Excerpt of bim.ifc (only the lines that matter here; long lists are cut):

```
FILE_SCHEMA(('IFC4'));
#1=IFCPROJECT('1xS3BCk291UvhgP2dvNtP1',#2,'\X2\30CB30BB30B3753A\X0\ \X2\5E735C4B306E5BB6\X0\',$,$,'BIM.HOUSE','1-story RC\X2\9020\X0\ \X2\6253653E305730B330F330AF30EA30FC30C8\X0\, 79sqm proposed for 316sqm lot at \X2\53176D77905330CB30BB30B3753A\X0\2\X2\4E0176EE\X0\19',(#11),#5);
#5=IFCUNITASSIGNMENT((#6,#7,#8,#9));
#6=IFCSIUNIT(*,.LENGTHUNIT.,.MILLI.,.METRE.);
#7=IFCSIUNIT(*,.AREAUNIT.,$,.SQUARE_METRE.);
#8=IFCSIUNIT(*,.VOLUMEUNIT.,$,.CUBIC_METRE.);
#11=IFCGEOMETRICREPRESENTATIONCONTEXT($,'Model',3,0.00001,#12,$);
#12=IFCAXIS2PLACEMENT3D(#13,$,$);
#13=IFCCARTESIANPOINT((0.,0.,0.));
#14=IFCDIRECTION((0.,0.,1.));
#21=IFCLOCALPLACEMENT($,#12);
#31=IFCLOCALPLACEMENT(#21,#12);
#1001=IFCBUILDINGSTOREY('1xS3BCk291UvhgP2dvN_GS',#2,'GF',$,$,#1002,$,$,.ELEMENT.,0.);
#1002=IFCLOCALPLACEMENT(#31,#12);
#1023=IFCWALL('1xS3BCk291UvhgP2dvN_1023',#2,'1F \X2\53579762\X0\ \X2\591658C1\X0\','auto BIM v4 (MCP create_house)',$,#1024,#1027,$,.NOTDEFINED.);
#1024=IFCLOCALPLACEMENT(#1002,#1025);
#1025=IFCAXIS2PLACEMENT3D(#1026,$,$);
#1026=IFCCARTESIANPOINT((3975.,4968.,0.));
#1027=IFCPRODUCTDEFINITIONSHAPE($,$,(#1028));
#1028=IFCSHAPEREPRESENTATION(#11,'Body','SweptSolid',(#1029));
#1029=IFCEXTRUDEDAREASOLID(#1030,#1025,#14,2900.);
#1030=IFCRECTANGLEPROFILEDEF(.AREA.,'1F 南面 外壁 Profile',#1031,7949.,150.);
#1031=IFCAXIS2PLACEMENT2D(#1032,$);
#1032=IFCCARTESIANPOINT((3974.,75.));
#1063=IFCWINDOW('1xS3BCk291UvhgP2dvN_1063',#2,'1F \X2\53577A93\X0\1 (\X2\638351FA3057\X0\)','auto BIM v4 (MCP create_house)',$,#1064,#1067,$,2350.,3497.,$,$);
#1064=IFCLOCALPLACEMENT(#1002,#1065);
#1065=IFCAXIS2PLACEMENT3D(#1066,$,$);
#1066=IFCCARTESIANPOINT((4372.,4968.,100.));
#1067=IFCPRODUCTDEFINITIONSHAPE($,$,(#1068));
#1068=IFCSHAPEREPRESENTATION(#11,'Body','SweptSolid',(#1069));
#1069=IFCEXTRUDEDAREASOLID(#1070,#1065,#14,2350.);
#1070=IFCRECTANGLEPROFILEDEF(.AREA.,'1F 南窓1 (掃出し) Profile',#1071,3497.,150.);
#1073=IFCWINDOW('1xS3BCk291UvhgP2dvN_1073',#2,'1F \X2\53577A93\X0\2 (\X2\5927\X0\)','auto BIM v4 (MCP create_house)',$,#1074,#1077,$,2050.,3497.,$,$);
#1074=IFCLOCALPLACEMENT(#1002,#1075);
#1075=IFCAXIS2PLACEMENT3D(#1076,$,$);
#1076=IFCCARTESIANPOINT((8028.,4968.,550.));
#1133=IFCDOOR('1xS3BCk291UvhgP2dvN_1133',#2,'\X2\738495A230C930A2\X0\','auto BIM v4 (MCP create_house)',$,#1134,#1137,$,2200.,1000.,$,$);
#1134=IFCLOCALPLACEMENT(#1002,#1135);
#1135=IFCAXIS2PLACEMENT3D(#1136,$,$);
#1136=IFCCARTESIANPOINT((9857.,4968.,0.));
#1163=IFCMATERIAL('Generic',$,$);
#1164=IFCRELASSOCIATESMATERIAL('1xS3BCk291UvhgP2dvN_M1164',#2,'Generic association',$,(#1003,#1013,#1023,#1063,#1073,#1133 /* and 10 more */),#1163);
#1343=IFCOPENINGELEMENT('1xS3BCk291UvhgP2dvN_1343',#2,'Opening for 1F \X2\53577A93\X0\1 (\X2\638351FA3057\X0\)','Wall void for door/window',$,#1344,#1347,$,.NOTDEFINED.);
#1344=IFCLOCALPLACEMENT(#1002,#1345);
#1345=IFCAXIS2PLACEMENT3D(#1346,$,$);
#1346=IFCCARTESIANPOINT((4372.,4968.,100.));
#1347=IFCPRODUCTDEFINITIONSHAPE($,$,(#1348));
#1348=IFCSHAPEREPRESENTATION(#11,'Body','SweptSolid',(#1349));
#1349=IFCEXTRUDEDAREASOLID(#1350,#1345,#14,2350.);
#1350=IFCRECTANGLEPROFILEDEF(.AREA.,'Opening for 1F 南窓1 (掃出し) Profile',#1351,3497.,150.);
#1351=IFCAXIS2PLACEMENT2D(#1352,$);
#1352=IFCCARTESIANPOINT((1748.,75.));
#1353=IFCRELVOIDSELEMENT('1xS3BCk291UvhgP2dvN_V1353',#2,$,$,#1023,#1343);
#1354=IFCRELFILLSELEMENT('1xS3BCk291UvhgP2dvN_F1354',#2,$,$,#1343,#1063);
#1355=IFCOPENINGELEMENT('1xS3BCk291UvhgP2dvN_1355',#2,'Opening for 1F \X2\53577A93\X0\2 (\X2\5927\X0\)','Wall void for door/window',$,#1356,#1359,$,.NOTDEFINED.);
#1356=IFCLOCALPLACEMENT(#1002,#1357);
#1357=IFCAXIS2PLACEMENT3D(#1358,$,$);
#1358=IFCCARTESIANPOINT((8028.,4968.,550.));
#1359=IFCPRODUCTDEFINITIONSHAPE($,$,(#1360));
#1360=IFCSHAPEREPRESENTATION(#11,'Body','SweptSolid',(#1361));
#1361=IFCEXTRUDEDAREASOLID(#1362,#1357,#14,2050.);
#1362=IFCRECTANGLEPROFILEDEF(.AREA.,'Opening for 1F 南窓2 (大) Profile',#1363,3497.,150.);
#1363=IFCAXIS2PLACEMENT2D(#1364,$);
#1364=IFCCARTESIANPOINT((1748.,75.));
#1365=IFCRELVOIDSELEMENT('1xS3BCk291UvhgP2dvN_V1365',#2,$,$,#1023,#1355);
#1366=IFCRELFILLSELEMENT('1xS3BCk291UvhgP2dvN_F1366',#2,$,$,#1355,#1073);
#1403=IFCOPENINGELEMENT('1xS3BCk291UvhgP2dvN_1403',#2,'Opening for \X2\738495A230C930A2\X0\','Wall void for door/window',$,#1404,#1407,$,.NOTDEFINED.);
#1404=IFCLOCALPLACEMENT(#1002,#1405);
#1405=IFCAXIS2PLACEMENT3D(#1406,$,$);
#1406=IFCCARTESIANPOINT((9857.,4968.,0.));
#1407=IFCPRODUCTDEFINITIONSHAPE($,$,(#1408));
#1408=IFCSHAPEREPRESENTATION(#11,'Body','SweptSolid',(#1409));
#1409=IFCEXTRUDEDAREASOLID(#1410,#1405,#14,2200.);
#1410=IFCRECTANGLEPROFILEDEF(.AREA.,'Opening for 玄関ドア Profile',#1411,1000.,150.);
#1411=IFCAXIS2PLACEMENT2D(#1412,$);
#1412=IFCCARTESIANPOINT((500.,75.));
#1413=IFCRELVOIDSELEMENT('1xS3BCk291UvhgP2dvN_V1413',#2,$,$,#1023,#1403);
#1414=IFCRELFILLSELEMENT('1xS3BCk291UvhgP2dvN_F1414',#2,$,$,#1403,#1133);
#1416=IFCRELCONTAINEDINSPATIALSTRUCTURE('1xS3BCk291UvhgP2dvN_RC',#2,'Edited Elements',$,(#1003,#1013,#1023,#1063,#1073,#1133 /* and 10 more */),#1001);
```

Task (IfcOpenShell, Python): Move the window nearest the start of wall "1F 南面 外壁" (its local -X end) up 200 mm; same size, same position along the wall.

```python
import numpy as np
import ifcopenshell
import ifcopenshell.api.geometry
import ifcopenshell.util.placement
import ifcopenshell.util.unit

model = ifcopenshell.open("bim.ifc")
unit_scale = ifcopenshell.util.unit.calculate_unit_scale(model)

window = model.by_guid("1xS3BCk291UvhgP2dvN_1063")
opening = window.FillsVoids[0].RelatingOpeningElement
dz = 0.2 / unit_scale

shift = np.array([0.0, 0.0, dz])
# The window is not placed relative to its opening, so move both.
for product in (opening, window):
    matrix = ifcopenshell.util.placement.get_local_placement(product.ObjectPlacement)
    matrix[:3, 3] += shift
    ifcopenshell.api.geometry.edit_object_placement(model, product=product, matrix=matrix, is_si=False)

print(f"moved by {dz * unit_scale:+.3f} m")

model.write("bim_rev.ifc")
```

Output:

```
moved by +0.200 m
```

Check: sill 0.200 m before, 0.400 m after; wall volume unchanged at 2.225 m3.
